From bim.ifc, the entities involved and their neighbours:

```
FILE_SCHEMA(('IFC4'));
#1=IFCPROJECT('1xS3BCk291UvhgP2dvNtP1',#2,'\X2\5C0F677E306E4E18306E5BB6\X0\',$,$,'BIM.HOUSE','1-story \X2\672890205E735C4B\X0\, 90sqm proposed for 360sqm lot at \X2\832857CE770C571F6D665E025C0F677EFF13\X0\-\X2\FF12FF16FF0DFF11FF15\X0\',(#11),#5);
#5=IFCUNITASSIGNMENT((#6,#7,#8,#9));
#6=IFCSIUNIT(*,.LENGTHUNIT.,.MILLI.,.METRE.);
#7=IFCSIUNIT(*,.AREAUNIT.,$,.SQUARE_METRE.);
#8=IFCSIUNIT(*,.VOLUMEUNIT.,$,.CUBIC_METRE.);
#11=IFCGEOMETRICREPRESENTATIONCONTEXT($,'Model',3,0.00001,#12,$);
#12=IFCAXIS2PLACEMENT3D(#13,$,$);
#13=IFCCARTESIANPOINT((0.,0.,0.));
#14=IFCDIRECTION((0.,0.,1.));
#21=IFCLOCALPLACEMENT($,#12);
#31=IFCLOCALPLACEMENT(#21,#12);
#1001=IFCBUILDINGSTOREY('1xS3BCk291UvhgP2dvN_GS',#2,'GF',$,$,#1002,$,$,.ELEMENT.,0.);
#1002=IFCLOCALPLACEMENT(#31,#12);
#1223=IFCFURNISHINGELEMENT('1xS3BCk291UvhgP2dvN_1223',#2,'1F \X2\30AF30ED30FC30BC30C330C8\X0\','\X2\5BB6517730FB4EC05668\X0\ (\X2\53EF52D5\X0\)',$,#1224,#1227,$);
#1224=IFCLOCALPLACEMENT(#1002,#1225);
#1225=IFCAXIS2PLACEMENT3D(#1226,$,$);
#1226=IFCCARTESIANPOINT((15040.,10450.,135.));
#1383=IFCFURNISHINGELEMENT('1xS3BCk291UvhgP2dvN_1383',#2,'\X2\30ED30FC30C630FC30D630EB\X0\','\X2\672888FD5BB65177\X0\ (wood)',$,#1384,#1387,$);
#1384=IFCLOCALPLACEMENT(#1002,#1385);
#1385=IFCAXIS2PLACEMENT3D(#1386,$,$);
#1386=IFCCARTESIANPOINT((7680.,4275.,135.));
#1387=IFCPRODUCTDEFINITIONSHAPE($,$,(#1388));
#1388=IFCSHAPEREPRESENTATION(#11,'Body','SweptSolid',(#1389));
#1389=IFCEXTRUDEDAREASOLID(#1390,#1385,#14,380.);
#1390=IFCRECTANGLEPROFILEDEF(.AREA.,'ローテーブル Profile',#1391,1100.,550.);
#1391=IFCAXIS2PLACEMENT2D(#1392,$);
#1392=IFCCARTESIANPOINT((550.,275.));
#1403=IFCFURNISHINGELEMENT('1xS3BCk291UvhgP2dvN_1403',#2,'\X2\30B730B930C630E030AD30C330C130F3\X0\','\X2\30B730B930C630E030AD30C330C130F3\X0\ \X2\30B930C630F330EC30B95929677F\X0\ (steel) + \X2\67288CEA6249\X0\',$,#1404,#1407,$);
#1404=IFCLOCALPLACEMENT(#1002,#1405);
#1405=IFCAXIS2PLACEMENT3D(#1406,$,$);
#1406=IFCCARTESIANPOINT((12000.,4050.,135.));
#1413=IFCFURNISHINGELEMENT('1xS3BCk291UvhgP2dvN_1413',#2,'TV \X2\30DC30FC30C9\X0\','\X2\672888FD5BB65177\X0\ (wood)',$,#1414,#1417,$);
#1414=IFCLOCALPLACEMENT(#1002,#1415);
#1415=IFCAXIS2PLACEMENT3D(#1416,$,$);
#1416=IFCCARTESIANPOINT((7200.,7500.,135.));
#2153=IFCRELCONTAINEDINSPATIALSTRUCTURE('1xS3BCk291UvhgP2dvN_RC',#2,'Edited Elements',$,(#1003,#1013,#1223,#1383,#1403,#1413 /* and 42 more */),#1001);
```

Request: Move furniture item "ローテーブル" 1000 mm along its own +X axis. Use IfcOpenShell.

```python
import ifcopenshell
import ifcopenshell.api.geometry
import ifcopenshell.util.placement

model = ifcopenshell.open("bim.ifc")

item = model.by_guid("1xS3BCk291UvhgP2dvN_1383")
matrix = ifcopenshell.util.placement.get_local_placement(item.ObjectPlacement)
matrix[:3, 3] += matrix[:3, 0] * 1000.0
ifcopenshell.api.geometry.edit_object_placement(model, product=item, matrix=matrix, is_si=False)

print(ifcopenshell.util.placement.get_local_placement(item.ObjectPlacement).round(3) + 0.0)

model.write("bim_v2.ifc")
```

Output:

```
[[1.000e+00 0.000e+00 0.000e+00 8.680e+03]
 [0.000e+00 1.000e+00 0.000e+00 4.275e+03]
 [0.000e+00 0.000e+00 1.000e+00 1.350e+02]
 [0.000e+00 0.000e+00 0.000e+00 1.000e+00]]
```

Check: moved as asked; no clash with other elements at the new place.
